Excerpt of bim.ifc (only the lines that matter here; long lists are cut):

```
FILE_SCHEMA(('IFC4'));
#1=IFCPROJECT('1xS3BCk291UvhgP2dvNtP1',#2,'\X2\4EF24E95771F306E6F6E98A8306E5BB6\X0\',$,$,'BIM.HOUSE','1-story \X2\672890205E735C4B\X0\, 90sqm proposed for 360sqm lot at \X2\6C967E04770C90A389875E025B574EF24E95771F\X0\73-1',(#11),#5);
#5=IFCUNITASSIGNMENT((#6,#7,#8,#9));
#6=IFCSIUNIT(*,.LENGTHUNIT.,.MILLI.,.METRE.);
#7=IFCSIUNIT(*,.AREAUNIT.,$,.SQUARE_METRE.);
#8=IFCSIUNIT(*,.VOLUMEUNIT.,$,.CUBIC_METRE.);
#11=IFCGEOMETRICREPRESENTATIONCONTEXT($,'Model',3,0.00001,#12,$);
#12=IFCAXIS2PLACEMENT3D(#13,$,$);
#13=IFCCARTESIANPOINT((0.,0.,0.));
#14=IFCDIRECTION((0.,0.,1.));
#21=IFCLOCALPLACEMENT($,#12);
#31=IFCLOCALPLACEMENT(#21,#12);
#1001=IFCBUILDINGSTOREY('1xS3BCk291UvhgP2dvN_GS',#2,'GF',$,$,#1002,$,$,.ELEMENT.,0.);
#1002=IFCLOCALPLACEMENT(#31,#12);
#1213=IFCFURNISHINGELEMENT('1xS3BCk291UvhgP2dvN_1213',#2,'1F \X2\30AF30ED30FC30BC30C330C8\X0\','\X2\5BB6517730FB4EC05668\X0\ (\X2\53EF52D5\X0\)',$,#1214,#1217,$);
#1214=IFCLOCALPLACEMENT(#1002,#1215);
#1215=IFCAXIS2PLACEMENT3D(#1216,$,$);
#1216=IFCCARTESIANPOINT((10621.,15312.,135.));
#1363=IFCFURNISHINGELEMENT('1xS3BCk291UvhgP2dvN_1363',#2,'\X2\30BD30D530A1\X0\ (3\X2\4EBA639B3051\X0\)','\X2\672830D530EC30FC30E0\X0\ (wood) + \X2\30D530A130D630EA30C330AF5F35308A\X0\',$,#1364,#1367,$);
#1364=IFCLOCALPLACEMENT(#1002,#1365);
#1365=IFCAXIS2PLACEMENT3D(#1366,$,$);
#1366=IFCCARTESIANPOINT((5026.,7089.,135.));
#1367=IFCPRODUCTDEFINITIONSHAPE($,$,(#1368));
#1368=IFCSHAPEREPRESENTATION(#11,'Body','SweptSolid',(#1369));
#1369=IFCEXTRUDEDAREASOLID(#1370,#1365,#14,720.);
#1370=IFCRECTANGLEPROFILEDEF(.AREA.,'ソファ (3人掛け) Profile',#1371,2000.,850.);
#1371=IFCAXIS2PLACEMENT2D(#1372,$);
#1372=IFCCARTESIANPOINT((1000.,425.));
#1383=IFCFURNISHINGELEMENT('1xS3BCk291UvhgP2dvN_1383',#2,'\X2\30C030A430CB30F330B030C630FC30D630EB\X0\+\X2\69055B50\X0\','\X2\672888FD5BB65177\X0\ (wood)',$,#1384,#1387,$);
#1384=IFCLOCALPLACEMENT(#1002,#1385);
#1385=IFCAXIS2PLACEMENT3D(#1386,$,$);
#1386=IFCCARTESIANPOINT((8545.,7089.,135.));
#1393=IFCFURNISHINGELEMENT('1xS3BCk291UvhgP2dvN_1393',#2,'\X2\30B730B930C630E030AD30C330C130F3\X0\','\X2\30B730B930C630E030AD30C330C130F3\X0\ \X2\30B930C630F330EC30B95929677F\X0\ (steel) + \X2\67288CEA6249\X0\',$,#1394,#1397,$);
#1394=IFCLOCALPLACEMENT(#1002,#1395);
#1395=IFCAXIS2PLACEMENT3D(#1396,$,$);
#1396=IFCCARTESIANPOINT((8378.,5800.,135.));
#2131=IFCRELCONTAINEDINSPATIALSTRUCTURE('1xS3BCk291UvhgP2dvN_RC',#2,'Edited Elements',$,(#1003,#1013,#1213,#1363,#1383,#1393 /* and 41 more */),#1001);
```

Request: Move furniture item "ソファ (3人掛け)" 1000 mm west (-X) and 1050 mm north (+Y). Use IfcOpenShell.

```python
import ifcopenshell
import ifcopenshell.api.geometry
import ifcopenshell.util.placement
import ifcopenshell.util.unit

model = ifcopenshell.open("bim.ifc")
unit_scale = ifcopenshell.util.unit.calculate_unit_scale(model)

item = model.by_guid("1xS3BCk291UvhgP2dvN_1363")
matrix = ifcopenshell.util.placement.get_local_placement(item.ObjectPlacement)
matrix[0, 3] -= 1 / unit_scale
matrix[1, 3] += 1.05 / unit_scale
ifcopenshell.api.geometry.edit_object_placement(model, product=item, matrix=matrix, is_si=False)

print(ifcopenshell.util.placement.get_local_placement(item.ObjectPlacement).round(3) + 0.0)

model.write("bim_edited.ifc")
```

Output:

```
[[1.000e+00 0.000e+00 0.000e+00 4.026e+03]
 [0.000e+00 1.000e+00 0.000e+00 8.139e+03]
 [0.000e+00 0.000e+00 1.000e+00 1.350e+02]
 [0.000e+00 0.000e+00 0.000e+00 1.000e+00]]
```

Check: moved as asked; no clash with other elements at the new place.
